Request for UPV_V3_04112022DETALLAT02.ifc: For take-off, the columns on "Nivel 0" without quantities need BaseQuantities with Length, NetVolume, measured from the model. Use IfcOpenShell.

First a look at what the model holds.

```python
import ifcopenshell
import ifcopenshell.util.element
import ifcopenshell.util.unit

model = ifcopenshell.open("UPV_V3_04112022DETALLAT02.ifc")
print(model.schema)
for unit_type in ("LENGTHUNIT", "AREAUNIT", "VOLUMEUNIT"):
    print(unit_type, ifcopenshell.util.unit.calculate_unit_scale(model, unit_type))
storey = next(s for s in model.by_type("IfcBuildingStorey") if s.Name == "Nivel 0")
columns = [e for e in ifcopenshell.util.element.get_decomposition(storey) if e.is_a("IfcColumn")]
for e in sorted(columns, key=lambda e: e.id()):
    print(e.id(), e.is_a(), e.Name, list(ifcopenshell.util.element.get_psets(e, qtos_only=True)), sep=" | ")
```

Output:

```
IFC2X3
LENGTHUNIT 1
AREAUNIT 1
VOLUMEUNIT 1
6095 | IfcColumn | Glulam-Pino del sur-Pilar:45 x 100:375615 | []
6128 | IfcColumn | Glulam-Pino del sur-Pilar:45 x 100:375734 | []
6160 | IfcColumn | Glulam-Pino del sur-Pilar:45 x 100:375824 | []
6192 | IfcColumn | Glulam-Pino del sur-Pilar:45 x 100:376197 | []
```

```python
import ifcopenshell
import ifcopenshell.api.pset
import ifcopenshell.geom
import ifcopenshell.util.element
import ifcopenshell.util.shape
import ifcopenshell.util.unit

model = ifcopenshell.open("UPV_V3_04112022DETALLAT02.ifc")
unit_scale = ifcopenshell.util.unit.calculate_unit_scale(model)
volume_scale = ifcopenshell.util.unit.calculate_unit_scale(model, "VOLUMEUNIT")
settings = ifcopenshell.geom.settings()

storey = next(s for s in model.by_type("IfcBuildingStorey") if s.Name == "Nivel 0")
columns = [e for e in ifcopenshell.util.element.get_decomposition(storey) if e.is_a("IfcColumn")]

for e in sorted(columns, key=lambda e: e.id()):
    if ifcopenshell.util.element.get_psets(e, qtos_only=True, should_inherit=False):
        continue
    # Geometry comes back in metres, in the element's own axes.
    shape = ifcopenshell.geom.create_shape(settings, e)
    values = {
        "Length": ifcopenshell.util.shape.get_z(shape.geometry) / unit_scale,
        "NetVolume": ifcopenshell.util.shape.get_volume(shape.geometry) / volume_scale,
    }
    qto = ifcopenshell.api.pset.add_qto(model, product=e, name="BaseQuantities")
    ifcopenshell.api.pset.edit_qto(model, qto=qto, properties=values)
    print(e.id(), {k: round(v, 3) for k, v in values.items()})

model.write("UPV_V3_04112022DETALLAT02_edited.ifc")
```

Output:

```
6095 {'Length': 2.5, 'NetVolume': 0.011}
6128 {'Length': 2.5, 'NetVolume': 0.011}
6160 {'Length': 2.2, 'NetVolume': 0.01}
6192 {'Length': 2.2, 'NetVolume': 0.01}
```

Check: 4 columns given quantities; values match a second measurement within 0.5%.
